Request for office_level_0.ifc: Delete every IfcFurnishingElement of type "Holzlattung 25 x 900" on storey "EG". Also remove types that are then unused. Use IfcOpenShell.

First a look at what the model holds.

```python
import ifcopenshell
import ifcopenshell.util.element

model = ifcopenshell.open("office_level_0.ifc")
print(model.schema)
storey = next(s for s in model.by_type("IfcBuildingStorey") if s.Name == "EG")
furniture = [e for e in ifcopenshell.util.element.get_decomposition(storey) if e.is_a("IfcFurnishingElement")]
seen = {}
for e in furniture:
    element_type = ifcopenshell.util.element.get_type(e)
    name = element_type.Name if element_type not in (None, e) else None
    seen[name] = seen.get(name, 0) + 1
for name, count in sorted(seen.items(), key=str):
    print(count, "x", name)
```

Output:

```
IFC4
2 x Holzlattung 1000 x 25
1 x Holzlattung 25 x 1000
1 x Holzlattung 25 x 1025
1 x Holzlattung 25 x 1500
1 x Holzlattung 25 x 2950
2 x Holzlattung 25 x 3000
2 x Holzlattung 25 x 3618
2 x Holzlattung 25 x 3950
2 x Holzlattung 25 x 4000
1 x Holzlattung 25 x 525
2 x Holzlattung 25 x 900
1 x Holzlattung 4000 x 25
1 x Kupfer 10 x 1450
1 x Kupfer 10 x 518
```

```python
import ifcopenshell
import ifcopenshell.api.root
import ifcopenshell.util.element

model = ifcopenshell.open("office_level_0.ifc")

storey = next(s for s in model.by_type("IfcBuildingStorey") if s.Name == "EG")
furniture = [e for e in ifcopenshell.util.element.get_decomposition(storey) if e.is_a("IfcFurnishingElement")]
targets = [e for e in furniture if (t := ifcopenshell.util.element.get_type(e)) not in (None, e) and t.Name == "Holzlattung 25 x 900"]
types = {ifcopenshell.util.element.get_type(e) for e in targets} - {None, *targets}

for e in targets:
    ifcopenshell.api.root.remove_product(model, product=e)
print(len(targets), "removed")

unused = [t for t in types if not ifcopenshell.util.element.get_types(t)]
for t in unused:
    ifcopenshell.api.root.remove_product(model, product=t)
print(len(unused), "unused types removed")

model.write("office_level_0-out.ifc")
```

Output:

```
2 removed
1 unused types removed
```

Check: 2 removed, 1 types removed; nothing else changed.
